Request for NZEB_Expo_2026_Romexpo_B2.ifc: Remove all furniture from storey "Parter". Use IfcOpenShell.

First a look at what the model holds.

```python
import ifcopenshell
import ifcopenshell.util.element

model = ifcopenshell.open("NZEB_Expo_2026_Romexpo_B2.ifc")
print(model.schema)
storey = next(s for s in model.by_type("IfcBuildingStorey") if s.Name == "Parter")
furniture = [e for e in ifcopenshell.util.element.get_decomposition(storey) if e.is_a("IfcFurnishingElement")]
seen = {}
for e in furniture:
    element_type = ifcopenshell.util.element.get_type(e)
    name = element_type.Name if element_type not in (None, e) else None
    seen[name] = seen.get(name, 0) + 1
for name, count in sorted(seen.items(), key=str):
    print(count, "x", name)
```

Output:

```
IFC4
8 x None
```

```python
import ifcopenshell
import ifcopenshell.api.root
import ifcopenshell.util.element

model = ifcopenshell.open("NZEB_Expo_2026_Romexpo_B2.ifc")

storey = next(s for s in model.by_type("IfcBuildingStorey") if s.Name == "Parter")
furniture = [e for e in ifcopenshell.util.element.get_decomposition(storey) if e.is_a("IfcFurnishingElement")]

for e in furniture:
    ifcopenshell.api.root.remove_product(model, product=e)
print(len(furniture), "removed")

model.write("NZEB_Expo_2026_Romexpo_B2-out.ifc")
```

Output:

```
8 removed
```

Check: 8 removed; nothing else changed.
